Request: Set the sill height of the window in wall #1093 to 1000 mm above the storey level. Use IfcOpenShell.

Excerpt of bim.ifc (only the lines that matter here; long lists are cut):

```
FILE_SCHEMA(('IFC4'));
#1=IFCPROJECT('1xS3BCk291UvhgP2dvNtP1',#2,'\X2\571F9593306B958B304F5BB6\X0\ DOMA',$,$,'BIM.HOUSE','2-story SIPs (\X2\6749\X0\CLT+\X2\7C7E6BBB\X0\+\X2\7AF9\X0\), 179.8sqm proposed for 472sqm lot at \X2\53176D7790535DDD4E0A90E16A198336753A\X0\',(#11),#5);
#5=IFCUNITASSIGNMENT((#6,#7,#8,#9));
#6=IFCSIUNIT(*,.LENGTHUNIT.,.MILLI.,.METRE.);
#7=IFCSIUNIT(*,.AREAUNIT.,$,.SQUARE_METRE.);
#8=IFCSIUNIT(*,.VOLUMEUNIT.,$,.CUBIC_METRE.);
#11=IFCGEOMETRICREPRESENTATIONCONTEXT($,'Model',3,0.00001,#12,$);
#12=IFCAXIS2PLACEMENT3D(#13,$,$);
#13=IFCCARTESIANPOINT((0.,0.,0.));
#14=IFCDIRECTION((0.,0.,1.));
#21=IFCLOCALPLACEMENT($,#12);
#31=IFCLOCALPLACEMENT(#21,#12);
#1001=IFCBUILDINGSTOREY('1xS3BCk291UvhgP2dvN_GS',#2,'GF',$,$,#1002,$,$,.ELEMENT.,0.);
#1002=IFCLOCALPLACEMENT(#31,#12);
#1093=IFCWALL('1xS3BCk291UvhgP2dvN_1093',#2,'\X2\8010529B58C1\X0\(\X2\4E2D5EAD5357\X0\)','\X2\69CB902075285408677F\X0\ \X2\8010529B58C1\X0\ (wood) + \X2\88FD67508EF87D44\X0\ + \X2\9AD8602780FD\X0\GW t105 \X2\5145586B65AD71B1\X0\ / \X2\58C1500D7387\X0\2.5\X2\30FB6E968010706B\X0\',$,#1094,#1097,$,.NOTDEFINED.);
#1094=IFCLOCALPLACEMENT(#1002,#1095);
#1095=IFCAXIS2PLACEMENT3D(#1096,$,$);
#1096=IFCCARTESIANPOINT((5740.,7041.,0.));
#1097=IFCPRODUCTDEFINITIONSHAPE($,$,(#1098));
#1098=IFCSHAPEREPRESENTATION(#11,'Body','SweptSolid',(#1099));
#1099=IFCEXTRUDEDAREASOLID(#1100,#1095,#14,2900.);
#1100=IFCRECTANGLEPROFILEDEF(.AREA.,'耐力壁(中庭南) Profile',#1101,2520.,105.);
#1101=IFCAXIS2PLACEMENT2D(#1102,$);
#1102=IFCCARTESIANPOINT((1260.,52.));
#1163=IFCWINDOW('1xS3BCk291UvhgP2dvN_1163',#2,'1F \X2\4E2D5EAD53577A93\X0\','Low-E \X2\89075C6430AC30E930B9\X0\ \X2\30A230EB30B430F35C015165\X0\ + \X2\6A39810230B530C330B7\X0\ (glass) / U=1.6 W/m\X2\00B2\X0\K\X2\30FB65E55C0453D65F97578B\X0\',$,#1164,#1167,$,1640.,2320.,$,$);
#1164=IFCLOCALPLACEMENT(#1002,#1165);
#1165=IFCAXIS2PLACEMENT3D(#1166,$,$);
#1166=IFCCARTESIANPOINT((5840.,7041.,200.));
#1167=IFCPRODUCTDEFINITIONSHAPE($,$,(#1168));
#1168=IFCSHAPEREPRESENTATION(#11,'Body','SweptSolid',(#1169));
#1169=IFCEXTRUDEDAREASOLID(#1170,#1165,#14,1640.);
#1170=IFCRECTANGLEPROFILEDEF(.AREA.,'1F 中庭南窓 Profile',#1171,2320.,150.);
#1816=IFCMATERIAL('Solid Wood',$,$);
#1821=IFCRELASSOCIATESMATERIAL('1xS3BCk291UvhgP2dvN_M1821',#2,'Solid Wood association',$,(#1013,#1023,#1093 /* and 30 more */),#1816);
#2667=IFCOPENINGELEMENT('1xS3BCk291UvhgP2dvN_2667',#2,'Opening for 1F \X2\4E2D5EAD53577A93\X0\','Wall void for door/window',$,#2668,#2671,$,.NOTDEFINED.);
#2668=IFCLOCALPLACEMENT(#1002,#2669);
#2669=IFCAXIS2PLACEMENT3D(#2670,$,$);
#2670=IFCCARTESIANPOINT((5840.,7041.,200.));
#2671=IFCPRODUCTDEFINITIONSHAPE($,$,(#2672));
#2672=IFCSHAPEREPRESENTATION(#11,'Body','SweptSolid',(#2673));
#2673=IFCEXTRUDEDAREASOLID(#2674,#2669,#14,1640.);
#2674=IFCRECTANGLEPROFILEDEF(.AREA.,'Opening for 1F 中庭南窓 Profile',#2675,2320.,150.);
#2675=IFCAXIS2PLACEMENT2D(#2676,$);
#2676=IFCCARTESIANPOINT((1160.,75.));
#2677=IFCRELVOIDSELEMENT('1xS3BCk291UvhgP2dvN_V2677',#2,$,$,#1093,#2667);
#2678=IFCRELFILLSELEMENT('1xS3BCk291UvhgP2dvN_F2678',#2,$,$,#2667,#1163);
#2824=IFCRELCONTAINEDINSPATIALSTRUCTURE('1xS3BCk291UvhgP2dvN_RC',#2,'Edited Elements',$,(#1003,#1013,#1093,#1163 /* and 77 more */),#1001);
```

```python
import numpy as np
import ifcopenshell
import ifcopenshell.api.geometry
import ifcopenshell.geom
import ifcopenshell.util.element
import ifcopenshell.util.placement
import ifcopenshell.util.shape
import ifcopenshell.util.unit

model = ifcopenshell.open("bim.ifc")
unit_scale = ifcopenshell.util.unit.calculate_unit_scale(model)

window = model.by_guid("1xS3BCk291UvhgP2dvN_1163")
opening = window.FillsVoids[0].RelatingOpeningElement
storey = ifcopenshell.util.element.get_container(window, ifc_class="IfcBuildingStorey")
level = ifcopenshell.util.placement.get_local_placement(storey.ObjectPlacement)[2, 3]

# The opening's origin need not be at the sill, so measure its lowest point.
shape = ifcopenshell.geom.create_shape(ifcopenshell.geom.settings(), opening)
bottom = ifcopenshell.util.shape.get_shape_bottom_elevation(shape, shape.geometry) / unit_scale
dz = level + 1000.0 - bottom

shift = np.array([0.0, 0.0, dz])
# The window is not placed relative to its opening, so move both.
for product in (opening, window):
    matrix = ifcopenshell.util.placement.get_local_placement(product.ObjectPlacement)
    matrix[:3, 3] += shift
    ifcopenshell.api.geometry.edit_object_placement(model, product=product, matrix=matrix, is_si=False)

print(f"moved by {dz * unit_scale:+.3f} m")

model.write("bim-out.ifc")
```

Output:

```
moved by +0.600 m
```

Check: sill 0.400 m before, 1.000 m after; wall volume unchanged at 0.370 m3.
